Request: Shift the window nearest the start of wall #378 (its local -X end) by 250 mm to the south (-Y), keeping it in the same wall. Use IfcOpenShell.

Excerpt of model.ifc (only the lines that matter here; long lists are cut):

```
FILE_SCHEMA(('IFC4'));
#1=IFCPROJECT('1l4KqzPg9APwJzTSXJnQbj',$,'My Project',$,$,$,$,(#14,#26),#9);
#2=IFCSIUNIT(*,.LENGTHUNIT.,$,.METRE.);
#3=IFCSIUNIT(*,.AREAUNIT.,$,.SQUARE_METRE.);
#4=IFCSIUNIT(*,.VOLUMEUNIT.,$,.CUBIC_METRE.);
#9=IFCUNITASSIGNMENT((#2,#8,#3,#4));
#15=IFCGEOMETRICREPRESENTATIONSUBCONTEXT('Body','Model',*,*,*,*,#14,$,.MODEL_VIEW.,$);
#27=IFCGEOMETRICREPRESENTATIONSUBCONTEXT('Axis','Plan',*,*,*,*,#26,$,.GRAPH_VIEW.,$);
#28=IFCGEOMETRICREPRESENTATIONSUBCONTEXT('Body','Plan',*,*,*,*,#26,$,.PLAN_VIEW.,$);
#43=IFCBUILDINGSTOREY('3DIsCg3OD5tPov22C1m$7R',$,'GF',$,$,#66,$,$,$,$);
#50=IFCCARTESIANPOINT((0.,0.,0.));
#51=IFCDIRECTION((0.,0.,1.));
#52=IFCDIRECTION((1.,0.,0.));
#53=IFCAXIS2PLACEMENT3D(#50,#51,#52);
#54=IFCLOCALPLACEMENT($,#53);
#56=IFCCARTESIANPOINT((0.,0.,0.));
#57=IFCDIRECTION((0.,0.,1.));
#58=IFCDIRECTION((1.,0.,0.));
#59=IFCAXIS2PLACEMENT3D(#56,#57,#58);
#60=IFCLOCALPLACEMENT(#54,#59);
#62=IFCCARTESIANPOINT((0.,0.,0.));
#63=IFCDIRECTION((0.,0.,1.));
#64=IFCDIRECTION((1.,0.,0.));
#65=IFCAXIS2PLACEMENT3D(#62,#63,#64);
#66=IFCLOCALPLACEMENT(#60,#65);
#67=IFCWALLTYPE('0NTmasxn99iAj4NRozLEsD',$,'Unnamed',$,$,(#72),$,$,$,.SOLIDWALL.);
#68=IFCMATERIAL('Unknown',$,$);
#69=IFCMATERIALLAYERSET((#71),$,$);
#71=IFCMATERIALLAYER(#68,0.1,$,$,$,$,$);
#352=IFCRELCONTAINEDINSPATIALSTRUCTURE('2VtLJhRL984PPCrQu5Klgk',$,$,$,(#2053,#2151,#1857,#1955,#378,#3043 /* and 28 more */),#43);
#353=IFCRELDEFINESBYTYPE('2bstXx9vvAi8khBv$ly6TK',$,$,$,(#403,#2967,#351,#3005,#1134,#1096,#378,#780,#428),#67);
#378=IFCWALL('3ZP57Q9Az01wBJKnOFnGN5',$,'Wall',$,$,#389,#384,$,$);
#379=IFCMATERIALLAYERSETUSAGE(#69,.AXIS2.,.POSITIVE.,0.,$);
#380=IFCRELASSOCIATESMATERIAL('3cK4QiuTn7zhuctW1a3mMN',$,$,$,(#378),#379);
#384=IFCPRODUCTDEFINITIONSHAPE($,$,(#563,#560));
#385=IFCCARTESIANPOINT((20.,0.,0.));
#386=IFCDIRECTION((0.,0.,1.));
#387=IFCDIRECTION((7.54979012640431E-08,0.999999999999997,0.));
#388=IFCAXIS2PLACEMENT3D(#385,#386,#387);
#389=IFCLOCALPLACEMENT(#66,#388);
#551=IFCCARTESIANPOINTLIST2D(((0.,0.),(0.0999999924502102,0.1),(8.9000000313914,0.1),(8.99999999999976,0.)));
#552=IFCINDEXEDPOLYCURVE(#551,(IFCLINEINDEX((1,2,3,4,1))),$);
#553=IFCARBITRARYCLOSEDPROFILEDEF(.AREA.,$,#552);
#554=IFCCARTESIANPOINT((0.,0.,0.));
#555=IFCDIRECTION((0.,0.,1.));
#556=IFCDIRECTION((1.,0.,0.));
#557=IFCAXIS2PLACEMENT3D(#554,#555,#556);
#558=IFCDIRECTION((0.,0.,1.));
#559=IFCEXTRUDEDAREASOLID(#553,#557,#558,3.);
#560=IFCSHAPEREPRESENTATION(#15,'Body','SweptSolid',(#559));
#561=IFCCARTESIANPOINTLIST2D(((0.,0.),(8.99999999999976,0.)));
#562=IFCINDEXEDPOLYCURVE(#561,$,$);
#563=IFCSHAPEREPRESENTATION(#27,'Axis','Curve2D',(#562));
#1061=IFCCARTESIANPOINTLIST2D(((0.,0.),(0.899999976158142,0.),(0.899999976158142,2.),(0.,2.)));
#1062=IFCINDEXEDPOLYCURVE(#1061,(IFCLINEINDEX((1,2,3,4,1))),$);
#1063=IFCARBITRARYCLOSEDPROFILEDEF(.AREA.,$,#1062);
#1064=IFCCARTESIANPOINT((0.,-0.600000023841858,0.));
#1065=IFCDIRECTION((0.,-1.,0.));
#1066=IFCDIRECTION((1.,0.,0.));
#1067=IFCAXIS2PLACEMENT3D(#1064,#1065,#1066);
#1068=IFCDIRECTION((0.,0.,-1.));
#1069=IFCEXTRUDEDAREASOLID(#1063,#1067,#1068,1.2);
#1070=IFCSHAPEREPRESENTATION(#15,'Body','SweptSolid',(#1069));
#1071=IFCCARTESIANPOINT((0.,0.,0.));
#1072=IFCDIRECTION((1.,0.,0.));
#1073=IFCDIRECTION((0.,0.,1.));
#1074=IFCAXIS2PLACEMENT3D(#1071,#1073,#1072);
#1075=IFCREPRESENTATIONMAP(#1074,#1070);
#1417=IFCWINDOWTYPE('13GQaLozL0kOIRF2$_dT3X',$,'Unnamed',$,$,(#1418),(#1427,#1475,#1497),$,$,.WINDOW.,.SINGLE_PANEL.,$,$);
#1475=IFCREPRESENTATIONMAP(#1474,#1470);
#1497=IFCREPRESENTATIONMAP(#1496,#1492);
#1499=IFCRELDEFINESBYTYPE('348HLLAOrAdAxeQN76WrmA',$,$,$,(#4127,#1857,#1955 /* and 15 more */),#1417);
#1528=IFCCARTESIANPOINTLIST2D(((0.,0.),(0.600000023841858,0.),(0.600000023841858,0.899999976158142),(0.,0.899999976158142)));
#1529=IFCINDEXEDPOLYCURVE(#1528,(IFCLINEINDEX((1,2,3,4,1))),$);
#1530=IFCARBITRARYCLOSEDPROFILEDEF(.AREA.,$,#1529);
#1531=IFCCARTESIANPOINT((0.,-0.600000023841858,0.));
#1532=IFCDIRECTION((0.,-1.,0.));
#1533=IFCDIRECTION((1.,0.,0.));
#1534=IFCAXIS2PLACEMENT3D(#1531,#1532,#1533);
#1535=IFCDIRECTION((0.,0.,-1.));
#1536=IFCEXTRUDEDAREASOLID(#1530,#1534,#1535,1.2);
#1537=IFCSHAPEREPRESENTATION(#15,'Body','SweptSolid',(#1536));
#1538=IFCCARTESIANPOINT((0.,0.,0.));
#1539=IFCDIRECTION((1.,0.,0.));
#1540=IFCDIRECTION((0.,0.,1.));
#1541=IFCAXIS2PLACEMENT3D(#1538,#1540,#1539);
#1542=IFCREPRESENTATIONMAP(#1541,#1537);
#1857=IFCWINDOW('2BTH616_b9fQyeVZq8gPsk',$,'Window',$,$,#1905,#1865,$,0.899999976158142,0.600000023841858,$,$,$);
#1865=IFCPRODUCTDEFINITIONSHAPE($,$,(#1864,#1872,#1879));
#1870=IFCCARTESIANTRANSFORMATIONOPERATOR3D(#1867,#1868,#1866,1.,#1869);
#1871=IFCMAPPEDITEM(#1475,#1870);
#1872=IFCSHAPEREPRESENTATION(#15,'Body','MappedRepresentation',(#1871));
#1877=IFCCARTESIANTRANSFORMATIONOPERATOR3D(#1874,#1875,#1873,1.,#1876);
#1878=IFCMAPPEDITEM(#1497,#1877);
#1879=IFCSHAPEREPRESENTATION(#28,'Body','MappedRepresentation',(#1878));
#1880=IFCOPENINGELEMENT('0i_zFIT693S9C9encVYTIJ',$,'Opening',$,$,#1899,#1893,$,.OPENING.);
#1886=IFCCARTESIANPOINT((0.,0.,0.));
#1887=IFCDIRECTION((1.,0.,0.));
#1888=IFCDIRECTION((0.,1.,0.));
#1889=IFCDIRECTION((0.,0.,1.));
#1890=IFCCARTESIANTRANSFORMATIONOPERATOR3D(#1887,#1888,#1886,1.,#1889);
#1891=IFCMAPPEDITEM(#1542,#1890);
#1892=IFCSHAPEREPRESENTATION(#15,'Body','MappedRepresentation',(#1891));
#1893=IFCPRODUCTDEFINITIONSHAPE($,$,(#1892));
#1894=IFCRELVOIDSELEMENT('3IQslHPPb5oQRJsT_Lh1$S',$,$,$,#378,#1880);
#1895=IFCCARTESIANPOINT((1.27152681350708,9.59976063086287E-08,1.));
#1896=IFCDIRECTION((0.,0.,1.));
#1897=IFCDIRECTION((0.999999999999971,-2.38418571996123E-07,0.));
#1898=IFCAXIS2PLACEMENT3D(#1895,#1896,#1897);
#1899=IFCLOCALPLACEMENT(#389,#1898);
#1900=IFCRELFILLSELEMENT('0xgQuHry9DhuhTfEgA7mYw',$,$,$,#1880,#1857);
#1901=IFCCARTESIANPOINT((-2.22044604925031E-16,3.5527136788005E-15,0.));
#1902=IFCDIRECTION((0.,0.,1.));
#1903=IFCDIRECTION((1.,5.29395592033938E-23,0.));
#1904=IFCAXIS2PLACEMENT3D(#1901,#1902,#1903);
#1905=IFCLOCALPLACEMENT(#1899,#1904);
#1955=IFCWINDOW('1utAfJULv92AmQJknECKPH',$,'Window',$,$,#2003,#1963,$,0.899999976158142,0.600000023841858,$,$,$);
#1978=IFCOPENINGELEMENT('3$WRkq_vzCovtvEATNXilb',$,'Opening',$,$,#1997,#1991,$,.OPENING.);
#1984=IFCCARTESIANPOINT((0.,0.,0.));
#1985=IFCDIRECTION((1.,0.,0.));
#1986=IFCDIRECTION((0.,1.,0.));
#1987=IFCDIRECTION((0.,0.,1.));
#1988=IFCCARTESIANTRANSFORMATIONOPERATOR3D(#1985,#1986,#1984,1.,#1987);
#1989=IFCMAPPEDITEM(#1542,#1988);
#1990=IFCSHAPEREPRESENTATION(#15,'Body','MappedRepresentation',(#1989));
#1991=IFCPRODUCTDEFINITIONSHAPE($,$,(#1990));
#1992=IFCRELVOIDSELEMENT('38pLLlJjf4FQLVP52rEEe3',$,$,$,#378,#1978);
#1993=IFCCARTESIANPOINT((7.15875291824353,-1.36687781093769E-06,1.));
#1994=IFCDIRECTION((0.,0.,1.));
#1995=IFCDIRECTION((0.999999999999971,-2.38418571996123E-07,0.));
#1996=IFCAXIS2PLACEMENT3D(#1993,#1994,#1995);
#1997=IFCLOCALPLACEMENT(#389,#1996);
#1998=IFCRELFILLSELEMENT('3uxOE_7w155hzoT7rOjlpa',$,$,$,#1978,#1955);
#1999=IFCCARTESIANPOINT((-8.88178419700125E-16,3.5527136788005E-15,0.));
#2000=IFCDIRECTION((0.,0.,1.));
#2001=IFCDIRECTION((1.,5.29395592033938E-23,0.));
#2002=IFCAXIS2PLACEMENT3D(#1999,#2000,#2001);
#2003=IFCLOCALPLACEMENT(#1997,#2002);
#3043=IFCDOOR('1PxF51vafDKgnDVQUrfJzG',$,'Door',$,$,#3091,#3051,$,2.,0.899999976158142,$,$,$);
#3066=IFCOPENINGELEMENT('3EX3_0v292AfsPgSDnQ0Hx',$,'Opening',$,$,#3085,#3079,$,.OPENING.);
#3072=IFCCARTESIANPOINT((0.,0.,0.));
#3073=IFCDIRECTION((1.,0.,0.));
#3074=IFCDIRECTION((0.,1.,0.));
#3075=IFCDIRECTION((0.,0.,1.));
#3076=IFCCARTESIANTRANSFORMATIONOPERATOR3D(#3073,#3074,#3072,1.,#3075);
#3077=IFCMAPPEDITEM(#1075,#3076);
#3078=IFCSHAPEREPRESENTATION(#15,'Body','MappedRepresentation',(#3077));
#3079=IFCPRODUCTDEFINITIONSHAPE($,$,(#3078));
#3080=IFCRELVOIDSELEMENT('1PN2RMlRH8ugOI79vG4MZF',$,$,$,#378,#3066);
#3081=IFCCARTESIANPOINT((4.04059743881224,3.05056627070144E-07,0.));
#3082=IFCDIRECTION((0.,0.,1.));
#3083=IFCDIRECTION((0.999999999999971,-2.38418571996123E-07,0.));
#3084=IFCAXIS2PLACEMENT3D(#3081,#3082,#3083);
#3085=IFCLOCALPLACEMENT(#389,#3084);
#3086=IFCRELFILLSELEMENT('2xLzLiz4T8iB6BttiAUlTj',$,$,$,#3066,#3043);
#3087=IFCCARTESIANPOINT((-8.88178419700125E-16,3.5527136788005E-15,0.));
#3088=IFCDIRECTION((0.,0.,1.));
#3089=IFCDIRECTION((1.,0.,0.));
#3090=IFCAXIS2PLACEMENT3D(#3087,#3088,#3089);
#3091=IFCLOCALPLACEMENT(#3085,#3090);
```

```python
import ifcopenshell
import ifcopenshell.api.geometry
import ifcopenshell.util.placement
import ifcopenshell.util.unit

model = ifcopenshell.open("model.ifc")
unit_scale = ifcopenshell.util.unit.calculate_unit_scale(model)

window = model.by_id(1857)
opening = window.FillsVoids[0].RelatingOpeningElement
wall = opening.VoidsElements[0].RelatingBuildingElement

wall_matrix = ifcopenshell.util.placement.get_local_placement(wall.ObjectPlacement)
shift = wall_matrix[:3, 0] * -0.25 / unit_scale
before = ifcopenshell.util.placement.get_local_placement(window.ObjectPlacement)[:3, 3].copy()

# The window is placed relative to its opening, so it follows when the opening moves.
matrix = ifcopenshell.util.placement.get_local_placement(opening.ObjectPlacement)
matrix[:3, 3] += shift
ifcopenshell.api.geometry.edit_object_placement(
    model, product=opening, matrix=matrix, is_si=False, should_transform_children=True
)

after = ifcopenshell.util.placement.get_local_placement(window.ObjectPlacement)[:3, 3]
print("window moved by", (after - before).round(3) + 0.0)

model.write("model_updated.ifc")
```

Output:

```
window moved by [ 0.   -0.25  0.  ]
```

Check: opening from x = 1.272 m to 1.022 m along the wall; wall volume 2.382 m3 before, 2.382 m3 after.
